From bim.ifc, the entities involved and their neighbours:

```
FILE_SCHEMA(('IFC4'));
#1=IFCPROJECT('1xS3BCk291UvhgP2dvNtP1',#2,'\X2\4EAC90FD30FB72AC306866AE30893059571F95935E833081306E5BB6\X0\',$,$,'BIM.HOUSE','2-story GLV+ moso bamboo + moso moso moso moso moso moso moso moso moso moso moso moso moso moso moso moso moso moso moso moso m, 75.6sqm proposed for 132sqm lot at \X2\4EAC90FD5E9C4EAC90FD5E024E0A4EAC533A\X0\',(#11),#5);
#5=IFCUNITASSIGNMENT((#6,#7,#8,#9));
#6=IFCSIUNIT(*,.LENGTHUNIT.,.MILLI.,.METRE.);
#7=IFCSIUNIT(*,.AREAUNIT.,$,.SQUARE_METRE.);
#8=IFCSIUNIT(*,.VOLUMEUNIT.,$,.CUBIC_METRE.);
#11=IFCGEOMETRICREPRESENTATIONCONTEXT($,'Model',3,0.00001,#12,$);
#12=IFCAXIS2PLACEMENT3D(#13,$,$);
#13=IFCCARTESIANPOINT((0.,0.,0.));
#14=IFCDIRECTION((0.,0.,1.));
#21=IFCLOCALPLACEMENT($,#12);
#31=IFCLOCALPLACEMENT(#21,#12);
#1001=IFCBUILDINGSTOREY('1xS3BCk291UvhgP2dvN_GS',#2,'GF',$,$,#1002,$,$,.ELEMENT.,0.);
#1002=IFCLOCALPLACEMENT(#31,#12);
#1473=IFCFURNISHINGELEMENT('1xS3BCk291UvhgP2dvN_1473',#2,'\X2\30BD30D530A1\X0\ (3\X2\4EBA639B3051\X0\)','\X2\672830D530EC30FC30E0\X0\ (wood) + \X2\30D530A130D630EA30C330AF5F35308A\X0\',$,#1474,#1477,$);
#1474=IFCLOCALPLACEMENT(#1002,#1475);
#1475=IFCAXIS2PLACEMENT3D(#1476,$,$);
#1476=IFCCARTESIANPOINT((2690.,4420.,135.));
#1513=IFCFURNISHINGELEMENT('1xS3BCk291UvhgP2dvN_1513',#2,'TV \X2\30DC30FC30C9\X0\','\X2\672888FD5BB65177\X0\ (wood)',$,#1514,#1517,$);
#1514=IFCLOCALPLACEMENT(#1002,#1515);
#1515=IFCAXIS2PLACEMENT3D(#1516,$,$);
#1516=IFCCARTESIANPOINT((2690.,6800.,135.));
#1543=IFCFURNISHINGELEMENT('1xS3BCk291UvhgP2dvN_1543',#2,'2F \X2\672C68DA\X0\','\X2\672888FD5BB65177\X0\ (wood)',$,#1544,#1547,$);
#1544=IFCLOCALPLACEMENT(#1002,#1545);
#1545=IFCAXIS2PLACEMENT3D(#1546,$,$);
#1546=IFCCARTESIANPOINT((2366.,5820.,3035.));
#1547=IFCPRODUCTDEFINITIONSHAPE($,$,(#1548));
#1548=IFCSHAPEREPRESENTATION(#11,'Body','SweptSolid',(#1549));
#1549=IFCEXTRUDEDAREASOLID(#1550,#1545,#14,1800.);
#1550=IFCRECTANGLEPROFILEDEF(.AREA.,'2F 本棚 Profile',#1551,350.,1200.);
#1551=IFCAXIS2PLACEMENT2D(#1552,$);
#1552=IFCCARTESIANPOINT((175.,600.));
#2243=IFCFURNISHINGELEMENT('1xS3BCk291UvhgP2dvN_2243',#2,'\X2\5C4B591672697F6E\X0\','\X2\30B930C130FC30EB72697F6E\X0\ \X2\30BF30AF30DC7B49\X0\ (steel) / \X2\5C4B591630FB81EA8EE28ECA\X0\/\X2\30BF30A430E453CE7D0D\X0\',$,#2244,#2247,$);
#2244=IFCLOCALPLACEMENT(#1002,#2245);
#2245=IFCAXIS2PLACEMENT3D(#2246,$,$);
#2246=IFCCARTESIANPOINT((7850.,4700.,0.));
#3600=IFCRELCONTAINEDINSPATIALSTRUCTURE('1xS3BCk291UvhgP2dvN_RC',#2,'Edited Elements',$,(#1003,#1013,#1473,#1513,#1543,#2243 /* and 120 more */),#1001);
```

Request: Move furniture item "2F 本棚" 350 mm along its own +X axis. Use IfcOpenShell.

```python
import ifcopenshell
import ifcopenshell.api.geometry
import ifcopenshell.util.placement

model = ifcopenshell.open("bim.ifc")

item = model.by_id(1543)
matrix = ifcopenshell.util.placement.get_local_placement(item.ObjectPlacement)
matrix[:3, 3] += matrix[:3, 0] * 350.0
ifcopenshell.api.geometry.edit_object_placement(model, product=item, matrix=matrix, is_si=False)

print(ifcopenshell.util.placement.get_local_placement(item.ObjectPlacement).round(3) + 0.0)

model.write("bim-out.ifc")
```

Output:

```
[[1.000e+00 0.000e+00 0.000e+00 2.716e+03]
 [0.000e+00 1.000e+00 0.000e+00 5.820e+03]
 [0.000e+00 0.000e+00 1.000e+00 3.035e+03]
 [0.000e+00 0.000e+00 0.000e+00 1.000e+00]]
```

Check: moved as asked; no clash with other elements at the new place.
